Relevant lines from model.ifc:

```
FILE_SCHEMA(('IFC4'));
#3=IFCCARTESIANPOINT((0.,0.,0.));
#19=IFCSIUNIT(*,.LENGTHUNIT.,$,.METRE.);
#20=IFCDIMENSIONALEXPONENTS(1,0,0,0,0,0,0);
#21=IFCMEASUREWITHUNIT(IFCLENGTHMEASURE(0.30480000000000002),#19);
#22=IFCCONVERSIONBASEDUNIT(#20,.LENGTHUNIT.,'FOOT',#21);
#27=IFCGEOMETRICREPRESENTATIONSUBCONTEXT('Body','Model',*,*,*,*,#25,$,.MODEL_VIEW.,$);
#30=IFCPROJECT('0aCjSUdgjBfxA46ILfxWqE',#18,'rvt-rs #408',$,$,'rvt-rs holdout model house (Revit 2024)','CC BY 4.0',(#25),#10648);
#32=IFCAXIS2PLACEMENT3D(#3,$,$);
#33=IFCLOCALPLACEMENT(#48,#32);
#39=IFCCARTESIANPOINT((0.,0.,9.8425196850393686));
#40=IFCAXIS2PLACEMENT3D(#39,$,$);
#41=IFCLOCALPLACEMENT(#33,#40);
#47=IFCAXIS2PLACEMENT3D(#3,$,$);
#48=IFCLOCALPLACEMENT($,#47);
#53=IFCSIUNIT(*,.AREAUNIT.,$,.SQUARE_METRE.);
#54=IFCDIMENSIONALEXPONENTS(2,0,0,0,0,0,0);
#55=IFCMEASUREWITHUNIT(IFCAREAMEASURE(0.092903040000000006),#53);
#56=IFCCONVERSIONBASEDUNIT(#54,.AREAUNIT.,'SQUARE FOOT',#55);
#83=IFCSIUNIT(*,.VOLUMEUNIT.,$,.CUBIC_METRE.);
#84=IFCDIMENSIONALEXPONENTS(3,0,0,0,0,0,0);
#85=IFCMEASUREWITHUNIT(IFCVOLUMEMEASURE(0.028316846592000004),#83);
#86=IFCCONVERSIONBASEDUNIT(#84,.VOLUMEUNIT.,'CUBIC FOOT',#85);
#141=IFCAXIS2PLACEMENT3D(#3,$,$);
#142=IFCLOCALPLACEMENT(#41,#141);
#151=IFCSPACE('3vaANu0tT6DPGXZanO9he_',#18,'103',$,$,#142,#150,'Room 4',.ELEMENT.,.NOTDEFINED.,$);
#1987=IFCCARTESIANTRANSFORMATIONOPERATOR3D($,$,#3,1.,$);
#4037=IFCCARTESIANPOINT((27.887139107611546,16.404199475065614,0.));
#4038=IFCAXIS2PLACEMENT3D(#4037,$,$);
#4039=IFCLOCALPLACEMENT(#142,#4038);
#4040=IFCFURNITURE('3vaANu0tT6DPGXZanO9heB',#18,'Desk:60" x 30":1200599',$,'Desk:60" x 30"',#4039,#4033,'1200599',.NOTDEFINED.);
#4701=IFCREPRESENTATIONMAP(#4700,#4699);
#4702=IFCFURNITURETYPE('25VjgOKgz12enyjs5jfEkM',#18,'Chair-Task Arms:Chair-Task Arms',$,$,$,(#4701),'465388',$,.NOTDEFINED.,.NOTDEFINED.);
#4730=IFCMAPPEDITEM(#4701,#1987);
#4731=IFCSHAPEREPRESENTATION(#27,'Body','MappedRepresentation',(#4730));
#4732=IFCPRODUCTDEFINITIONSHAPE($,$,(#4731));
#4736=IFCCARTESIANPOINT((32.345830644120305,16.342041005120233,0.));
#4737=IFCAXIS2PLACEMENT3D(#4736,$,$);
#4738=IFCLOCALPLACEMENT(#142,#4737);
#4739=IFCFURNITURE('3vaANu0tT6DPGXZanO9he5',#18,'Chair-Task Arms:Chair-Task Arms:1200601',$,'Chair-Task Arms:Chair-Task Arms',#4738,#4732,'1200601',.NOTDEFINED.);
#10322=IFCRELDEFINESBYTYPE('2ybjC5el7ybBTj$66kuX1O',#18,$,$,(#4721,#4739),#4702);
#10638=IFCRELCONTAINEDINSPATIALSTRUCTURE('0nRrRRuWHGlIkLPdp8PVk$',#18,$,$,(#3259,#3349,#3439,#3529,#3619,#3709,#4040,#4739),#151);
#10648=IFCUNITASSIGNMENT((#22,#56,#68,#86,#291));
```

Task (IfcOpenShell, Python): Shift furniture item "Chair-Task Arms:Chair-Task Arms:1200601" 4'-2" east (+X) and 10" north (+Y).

```python
import ifcopenshell
import ifcopenshell.api.geometry
import ifcopenshell.util.placement
import ifcopenshell.util.unit

model = ifcopenshell.open("model.ifc")
unit_scale = ifcopenshell.util.unit.calculate_unit_scale(model)

item = model.by_id(4739)
matrix = ifcopenshell.util.placement.get_local_placement(item.ObjectPlacement)
matrix[0, 3] += 50 * 0.0254 / unit_scale
matrix[1, 3] += 10 * 0.0254 / unit_scale
ifcopenshell.api.geometry.edit_object_placement(model, product=item, matrix=matrix, is_si=False)

print(ifcopenshell.util.placement.get_local_placement(item.ObjectPlacement).round(3) + 0.0)

model.write("model_updated.ifc")
```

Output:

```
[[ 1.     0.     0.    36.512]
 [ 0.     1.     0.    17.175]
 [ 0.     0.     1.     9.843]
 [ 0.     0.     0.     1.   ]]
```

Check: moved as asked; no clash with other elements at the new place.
